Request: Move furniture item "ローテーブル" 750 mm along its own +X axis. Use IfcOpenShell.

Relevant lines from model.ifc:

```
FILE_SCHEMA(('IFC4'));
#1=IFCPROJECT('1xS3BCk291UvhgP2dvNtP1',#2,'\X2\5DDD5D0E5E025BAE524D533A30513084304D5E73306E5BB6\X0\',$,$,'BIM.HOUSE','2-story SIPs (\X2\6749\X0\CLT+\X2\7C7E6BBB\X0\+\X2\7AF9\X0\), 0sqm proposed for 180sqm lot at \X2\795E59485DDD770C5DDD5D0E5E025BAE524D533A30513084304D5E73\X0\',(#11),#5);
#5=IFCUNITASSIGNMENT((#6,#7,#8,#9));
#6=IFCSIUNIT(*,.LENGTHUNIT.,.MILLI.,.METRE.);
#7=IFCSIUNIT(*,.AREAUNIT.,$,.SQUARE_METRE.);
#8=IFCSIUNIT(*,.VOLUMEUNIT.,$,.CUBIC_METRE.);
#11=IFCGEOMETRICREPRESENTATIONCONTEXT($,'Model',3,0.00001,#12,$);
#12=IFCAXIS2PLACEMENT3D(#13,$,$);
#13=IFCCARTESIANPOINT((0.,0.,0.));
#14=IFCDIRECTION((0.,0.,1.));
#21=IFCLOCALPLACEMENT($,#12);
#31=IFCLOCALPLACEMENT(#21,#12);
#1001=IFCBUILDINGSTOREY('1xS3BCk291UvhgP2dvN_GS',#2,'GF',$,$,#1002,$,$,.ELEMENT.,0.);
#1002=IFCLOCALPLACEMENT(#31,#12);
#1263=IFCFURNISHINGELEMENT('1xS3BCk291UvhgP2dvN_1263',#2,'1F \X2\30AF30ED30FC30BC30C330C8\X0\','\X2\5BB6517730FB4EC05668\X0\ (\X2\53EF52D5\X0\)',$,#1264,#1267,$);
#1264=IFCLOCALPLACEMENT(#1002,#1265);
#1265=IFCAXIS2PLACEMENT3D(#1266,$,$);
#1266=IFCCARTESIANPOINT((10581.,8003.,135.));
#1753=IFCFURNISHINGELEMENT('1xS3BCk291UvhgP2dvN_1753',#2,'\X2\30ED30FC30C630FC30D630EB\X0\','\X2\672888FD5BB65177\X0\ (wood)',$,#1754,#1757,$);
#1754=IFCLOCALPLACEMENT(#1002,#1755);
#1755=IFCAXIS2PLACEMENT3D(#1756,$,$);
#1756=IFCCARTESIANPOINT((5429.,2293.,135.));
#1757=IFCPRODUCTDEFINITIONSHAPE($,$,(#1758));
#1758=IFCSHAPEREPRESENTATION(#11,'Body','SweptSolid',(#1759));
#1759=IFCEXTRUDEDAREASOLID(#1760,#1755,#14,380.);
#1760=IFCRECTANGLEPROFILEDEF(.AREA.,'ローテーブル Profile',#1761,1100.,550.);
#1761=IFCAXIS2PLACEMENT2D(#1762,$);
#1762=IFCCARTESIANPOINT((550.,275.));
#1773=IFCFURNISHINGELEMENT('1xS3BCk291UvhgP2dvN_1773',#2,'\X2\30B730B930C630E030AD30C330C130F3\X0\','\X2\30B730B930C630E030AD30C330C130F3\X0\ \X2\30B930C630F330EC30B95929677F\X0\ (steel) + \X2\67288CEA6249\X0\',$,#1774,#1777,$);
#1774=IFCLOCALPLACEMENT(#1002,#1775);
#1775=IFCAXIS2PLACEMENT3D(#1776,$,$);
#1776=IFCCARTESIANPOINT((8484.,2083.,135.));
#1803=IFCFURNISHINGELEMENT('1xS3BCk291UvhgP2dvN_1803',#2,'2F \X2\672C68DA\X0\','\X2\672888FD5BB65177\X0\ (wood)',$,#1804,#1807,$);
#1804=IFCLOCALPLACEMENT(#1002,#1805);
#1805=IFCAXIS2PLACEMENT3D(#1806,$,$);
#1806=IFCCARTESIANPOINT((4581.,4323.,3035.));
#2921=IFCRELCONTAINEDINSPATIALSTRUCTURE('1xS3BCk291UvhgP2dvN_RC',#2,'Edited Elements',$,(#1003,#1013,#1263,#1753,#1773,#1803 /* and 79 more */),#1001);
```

```python
import ifcopenshell
import ifcopenshell.api.geometry
import ifcopenshell.util.placement

model = ifcopenshell.open("model.ifc")

item = model.by_guid("1xS3BCk291UvhgP2dvN_1753")
matrix = ifcopenshell.util.placement.get_local_placement(item.ObjectPlacement)
matrix[:3, 3] += matrix[:3, 0] * 750.0
ifcopenshell.api.geometry.edit_object_placement(model, product=item, matrix=matrix, is_si=False)

print(ifcopenshell.util.placement.get_local_placement(item.ObjectPlacement).round(3) + 0.0)

model.write("model-out.ifc")
```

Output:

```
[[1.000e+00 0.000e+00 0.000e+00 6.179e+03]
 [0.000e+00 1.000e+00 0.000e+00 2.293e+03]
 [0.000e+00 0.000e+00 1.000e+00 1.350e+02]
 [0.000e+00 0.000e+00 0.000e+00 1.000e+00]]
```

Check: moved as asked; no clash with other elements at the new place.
